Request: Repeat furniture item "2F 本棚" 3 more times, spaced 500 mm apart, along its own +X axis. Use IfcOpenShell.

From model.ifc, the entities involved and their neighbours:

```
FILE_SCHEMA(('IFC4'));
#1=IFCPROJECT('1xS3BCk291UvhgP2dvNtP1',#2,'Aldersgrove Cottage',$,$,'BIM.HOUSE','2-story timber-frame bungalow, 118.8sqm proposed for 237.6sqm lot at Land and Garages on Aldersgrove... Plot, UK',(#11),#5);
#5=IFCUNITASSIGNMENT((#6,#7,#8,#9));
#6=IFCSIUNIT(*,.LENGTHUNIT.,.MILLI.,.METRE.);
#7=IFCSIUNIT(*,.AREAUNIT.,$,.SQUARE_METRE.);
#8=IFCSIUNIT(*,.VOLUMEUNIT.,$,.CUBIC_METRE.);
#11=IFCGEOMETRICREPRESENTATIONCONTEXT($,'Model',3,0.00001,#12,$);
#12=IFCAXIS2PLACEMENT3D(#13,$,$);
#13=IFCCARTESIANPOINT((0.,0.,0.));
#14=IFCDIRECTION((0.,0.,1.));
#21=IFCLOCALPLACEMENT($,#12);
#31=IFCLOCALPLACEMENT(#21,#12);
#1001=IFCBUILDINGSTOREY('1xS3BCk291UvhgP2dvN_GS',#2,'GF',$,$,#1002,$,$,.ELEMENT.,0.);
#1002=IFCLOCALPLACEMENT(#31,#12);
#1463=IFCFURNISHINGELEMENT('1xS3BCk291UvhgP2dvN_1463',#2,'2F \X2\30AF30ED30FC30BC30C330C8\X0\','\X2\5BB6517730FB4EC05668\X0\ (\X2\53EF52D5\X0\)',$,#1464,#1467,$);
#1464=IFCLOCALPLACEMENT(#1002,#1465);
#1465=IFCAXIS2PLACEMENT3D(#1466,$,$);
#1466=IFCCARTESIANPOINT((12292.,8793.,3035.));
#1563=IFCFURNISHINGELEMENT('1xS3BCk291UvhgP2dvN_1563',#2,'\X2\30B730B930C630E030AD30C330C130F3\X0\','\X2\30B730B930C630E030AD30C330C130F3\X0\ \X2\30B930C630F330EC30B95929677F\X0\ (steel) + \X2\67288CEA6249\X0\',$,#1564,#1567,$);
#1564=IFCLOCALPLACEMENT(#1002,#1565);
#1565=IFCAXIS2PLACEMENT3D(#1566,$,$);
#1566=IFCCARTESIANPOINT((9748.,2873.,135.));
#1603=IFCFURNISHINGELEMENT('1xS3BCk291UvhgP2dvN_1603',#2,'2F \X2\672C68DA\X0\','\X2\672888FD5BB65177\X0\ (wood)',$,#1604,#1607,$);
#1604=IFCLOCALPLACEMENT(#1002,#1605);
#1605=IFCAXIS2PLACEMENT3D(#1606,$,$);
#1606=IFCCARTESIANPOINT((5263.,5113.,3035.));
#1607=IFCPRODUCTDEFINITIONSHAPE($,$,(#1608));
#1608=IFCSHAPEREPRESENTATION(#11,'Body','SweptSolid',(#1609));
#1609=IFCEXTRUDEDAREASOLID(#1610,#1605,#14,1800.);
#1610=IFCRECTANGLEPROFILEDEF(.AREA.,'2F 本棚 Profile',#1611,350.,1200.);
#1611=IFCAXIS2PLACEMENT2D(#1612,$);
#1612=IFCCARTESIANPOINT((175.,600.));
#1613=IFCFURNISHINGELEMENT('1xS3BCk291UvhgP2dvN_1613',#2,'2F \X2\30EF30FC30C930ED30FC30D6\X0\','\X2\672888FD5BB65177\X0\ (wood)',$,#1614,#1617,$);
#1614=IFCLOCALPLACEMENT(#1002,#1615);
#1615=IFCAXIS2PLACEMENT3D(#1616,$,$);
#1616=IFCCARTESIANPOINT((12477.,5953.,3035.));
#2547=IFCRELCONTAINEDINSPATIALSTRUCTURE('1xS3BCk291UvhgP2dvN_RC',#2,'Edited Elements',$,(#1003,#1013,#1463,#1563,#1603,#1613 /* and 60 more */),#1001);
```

```python
import ifcopenshell
import ifcopenshell.api.geometry
import ifcopenshell.api.root
import ifcopenshell.util.element
import ifcopenshell.util.placement

model = ifcopenshell.open("model.ifc")


def reuse_history(source, copy):
    """copy_class also copies each property set's owner history, people and application; keep the originals."""
    for rel in copy.IsDefinedBy:
        if rel.is_a("IfcRelDefinesByProperties") and (history := rel.RelatingPropertyDefinition.OwnerHistory):
            rel.RelatingPropertyDefinition.OwnerHistory = source.OwnerHistory
            ifcopenshell.util.element.remove_deep2(model, history)


source = model.by_guid("1xS3BCk291UvhgP2dvN_1603")
base = ifcopenshell.util.placement.get_local_placement(source.ObjectPlacement)
step = base[:3, 0] * 500.0

for i in range(1, 4):
    copy = ifcopenshell.api.root.copy_class(model, product=source)
    copy.Representation = ifcopenshell.util.element.copy_deep(
        model, source.Representation, exclude=["IfcGeometricRepresentationContext", "IfcRepresentationMap"]
    )
    reuse_history(source, copy)
    matrix = base.copy()
    matrix[:3, 3] += i * step
    print("added at", matrix[:3, 3].round(3) + 0.0)
    ifcopenshell.api.geometry.edit_object_placement(model, product=copy, matrix=matrix, is_si=False)

model.write("model_v2.ifc")
```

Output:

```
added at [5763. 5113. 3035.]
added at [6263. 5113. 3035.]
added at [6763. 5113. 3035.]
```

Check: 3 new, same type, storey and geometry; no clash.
